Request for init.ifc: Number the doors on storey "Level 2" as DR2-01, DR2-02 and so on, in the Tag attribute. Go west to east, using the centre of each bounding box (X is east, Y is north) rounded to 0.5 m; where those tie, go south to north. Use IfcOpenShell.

First a look at what the model holds.

```python
import ifcopenshell
import ifcopenshell.util.element
import ifcopenshell.util.placement

model = ifcopenshell.open("init.ifc")
print(model.schema)
storey = next(s for s in model.by_type("IfcBuildingStorey") if s.Name == "Level 2")
doors = [e for e in ifcopenshell.util.element.get_decomposition(storey) if e.is_a("IfcDoor")]
for e in sorted(doors, key=lambda e: e.id()):
    origin = ifcopenshell.util.placement.get_local_placement(e.ObjectPlacement)[:3, 3]
    print(e.id(), e.Tag, e.Name, origin.round(2) + 0.0, sep=" | ")
```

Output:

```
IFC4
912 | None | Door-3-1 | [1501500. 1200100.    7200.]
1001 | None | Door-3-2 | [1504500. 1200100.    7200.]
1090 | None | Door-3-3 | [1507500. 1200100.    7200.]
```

```python
import ifcopenshell
import ifcopenshell.geom
import ifcopenshell.util.element
import ifcopenshell.util.shape

model = ifcopenshell.open("init.ifc")
settings = ifcopenshell.geom.settings()
settings.set("use-world-coords", True)


def centre(element):
    shape = ifcopenshell.geom.create_shape(settings, element)
    return ifcopenshell.util.shape.get_bbox_centroid(shape.geometry)


storey = next(s for s in model.by_type("IfcBuildingStorey") if s.Name == "Level 2")
doors = [e for e in ifcopenshell.util.element.get_decomposition(storey) if e.is_a("IfcDoor")]

# Insertion points can sit at a corner or the storey origin, so sort by the geometry (in metres).
centres = {e: centre(e) for e in doors}
doors.sort(key=lambda e: (round(centres[e][0] / 0.5), centres[e][1]))

for i, e in enumerate(doors, start=1):
    number = f"DR2-{i:02d}"
    e.Tag = number
    print(e.id(), number)

model.write("init_updated.ifc")
```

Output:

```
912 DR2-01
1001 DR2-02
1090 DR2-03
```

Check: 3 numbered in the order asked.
